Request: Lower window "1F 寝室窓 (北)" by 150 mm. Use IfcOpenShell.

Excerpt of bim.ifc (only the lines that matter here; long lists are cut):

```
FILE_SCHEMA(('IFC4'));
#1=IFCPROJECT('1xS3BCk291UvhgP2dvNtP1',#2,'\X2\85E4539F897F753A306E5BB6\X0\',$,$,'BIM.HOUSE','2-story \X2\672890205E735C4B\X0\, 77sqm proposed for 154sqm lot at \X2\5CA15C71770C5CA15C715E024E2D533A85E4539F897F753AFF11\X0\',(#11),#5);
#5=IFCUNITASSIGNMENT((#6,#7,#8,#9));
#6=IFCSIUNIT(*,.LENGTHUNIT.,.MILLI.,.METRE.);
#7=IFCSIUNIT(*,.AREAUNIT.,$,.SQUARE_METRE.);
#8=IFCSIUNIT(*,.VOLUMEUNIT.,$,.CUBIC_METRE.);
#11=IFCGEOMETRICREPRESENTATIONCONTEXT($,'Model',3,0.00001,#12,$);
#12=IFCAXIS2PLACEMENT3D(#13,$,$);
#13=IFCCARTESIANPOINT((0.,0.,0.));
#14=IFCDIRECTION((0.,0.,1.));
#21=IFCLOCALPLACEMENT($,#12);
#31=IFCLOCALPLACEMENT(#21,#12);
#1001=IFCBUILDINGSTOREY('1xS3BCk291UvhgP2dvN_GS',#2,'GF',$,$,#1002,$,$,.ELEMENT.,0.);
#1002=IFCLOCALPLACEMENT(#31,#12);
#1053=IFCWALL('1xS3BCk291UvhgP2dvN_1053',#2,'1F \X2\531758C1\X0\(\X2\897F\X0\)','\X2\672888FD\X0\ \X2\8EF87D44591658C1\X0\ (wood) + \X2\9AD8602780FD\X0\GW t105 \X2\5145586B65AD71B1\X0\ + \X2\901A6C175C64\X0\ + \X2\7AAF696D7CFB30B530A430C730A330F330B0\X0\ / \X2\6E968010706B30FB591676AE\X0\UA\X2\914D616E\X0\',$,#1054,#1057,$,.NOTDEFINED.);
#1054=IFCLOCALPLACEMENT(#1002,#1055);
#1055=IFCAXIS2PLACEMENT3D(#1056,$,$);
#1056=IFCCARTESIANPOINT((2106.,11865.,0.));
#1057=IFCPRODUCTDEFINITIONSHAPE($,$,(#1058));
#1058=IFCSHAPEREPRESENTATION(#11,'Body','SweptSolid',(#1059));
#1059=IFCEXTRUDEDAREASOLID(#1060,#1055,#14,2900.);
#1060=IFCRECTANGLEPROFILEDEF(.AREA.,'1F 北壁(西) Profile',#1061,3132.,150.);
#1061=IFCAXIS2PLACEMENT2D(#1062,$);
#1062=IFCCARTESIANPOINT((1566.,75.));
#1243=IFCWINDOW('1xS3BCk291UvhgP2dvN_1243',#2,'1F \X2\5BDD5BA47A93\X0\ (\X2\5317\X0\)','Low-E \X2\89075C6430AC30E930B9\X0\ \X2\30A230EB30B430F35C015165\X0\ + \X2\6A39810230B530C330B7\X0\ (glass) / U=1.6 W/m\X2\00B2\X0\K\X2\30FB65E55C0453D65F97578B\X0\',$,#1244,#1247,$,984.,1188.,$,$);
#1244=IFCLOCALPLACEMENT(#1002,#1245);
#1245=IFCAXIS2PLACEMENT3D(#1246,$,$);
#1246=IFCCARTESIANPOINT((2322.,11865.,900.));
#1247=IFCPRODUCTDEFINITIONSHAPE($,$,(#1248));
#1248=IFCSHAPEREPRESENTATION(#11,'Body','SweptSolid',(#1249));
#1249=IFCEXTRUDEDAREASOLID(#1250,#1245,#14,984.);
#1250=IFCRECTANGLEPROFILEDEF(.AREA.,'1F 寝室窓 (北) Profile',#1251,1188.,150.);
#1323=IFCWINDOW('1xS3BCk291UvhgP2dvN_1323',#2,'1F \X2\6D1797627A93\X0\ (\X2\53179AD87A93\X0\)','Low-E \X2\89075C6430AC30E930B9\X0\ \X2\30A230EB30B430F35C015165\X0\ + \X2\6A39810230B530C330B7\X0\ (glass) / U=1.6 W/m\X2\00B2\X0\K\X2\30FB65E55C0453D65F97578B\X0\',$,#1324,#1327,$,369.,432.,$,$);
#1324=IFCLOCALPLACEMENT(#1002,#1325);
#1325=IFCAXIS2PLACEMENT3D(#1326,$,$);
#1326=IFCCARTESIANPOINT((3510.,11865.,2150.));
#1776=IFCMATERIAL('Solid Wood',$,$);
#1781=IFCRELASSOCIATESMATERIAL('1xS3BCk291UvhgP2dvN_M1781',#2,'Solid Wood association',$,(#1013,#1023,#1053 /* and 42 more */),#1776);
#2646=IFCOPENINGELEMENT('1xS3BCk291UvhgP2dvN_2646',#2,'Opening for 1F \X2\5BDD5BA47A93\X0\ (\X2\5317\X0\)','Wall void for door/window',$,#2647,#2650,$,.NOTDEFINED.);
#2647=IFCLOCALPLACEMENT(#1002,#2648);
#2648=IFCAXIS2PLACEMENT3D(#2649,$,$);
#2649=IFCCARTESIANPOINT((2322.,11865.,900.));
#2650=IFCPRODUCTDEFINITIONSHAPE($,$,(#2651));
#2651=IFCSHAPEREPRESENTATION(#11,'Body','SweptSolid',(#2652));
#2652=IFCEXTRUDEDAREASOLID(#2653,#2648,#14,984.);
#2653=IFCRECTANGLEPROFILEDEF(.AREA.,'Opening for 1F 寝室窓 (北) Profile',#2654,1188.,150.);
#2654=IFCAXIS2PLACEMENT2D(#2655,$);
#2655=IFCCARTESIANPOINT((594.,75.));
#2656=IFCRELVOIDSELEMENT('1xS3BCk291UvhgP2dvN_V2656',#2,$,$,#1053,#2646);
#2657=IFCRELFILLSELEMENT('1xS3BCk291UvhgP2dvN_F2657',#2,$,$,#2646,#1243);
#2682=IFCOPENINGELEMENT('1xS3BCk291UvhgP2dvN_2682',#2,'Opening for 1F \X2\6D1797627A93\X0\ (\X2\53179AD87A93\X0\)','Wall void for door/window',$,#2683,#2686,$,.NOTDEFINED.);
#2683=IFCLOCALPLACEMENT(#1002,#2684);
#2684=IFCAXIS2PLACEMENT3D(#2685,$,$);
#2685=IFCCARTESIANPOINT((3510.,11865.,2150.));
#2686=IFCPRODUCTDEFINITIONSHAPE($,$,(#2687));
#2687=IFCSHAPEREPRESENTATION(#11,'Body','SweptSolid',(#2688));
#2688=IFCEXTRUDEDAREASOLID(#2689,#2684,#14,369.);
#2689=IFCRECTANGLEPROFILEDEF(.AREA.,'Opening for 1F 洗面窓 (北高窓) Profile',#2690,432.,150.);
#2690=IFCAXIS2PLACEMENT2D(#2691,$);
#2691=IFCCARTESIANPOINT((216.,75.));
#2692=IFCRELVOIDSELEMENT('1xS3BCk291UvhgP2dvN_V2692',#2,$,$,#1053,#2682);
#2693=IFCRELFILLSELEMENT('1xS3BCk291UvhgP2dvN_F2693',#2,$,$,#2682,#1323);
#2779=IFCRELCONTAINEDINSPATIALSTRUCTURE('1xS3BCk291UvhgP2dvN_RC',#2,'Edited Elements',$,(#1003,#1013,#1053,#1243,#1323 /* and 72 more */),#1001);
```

```python
import numpy as np
import ifcopenshell
import ifcopenshell.api.geometry
import ifcopenshell.util.placement
import ifcopenshell.util.unit

model = ifcopenshell.open("bim.ifc")
unit_scale = ifcopenshell.util.unit.calculate_unit_scale(model)

window = model.by_guid("1xS3BCk291UvhgP2dvN_1243")
opening = window.FillsVoids[0].RelatingOpeningElement
dz = -0.15 / unit_scale

shift = np.array([0.0, 0.0, dz])
# The window is not placed relative to its opening, so move both.
for product in (opening, window):
    matrix = ifcopenshell.util.placement.get_local_placement(product.ObjectPlacement)
    matrix[:3, 3] += shift
    ifcopenshell.api.geometry.edit_object_placement(model, product=product, matrix=matrix, is_si=False)

print(f"moved by {dz * unit_scale:+.3f} m")

model.write("bim-out.ifc")
```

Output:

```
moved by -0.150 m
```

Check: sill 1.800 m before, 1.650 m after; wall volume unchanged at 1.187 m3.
